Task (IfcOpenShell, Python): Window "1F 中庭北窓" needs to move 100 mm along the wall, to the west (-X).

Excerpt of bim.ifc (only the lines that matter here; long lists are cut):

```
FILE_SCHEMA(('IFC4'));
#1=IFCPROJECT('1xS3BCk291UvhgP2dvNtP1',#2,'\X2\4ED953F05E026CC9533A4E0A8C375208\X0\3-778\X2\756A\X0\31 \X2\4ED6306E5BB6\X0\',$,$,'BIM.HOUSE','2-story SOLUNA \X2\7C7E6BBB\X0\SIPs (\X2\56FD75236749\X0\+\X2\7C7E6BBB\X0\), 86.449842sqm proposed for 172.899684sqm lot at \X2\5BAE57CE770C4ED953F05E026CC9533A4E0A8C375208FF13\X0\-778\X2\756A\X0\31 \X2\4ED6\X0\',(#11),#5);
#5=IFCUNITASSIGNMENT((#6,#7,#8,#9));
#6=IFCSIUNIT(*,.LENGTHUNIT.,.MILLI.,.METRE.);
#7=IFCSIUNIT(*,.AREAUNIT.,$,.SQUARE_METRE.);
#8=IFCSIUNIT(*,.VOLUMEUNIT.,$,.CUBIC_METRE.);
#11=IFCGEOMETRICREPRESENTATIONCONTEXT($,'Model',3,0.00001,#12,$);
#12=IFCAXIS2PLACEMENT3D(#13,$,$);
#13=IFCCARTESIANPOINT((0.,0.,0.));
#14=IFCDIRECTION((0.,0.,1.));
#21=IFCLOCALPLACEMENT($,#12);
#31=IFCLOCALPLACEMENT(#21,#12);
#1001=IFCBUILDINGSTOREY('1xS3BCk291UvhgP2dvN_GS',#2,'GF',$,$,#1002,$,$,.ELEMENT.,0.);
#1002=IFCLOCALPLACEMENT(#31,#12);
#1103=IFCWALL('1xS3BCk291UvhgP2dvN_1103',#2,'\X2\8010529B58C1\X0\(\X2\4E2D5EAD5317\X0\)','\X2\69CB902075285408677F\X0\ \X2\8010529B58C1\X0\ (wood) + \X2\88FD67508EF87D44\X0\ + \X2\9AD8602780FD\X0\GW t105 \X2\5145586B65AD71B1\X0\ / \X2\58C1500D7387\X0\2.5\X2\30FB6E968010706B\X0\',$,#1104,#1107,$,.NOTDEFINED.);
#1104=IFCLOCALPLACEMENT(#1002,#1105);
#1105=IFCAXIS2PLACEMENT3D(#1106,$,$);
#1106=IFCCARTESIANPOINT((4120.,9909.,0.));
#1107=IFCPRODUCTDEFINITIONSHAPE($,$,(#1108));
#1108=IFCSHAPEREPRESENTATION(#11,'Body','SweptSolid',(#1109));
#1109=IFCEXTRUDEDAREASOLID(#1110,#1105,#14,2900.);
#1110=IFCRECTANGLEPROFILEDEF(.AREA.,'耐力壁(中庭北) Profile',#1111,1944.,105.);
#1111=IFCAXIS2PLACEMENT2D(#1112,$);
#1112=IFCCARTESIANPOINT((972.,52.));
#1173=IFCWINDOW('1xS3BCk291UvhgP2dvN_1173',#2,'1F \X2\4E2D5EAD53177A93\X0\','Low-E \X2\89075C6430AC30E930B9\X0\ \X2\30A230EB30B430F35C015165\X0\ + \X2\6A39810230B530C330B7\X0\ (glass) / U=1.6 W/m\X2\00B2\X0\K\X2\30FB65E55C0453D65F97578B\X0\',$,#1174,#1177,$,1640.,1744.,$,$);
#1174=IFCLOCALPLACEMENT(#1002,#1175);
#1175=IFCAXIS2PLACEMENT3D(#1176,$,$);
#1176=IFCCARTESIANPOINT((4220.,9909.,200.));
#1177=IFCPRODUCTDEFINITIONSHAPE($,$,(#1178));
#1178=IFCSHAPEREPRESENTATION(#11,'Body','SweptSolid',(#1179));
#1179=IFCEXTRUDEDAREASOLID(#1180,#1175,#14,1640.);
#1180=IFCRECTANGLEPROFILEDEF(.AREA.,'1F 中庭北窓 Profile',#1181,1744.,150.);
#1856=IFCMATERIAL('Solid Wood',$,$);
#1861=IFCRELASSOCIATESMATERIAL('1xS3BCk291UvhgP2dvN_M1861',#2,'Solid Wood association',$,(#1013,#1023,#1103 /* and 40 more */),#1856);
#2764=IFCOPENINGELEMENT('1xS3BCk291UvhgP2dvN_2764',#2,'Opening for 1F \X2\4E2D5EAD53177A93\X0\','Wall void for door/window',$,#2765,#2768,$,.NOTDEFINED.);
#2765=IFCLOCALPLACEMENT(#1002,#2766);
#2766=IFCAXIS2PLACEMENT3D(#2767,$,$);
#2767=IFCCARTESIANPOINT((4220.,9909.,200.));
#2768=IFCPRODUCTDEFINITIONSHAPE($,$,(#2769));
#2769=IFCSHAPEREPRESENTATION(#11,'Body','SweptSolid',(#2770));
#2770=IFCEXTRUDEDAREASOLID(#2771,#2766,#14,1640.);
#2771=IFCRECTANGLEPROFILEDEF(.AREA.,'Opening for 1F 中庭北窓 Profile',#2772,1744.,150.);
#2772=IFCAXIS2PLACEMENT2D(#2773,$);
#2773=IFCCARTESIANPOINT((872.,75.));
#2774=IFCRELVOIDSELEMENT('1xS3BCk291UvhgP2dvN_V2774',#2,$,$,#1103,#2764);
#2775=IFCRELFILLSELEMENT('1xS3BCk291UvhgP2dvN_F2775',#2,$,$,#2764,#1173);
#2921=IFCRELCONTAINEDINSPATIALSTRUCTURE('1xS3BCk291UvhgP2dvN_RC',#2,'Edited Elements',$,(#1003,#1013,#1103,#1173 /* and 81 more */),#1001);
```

```python
import ifcopenshell
import ifcopenshell.api.geometry
import ifcopenshell.util.placement
import ifcopenshell.util.unit

model = ifcopenshell.open("bim.ifc")
unit_scale = ifcopenshell.util.unit.calculate_unit_scale(model)

window = model.by_guid("1xS3BCk291UvhgP2dvN_1173")
opening = window.FillsVoids[0].RelatingOpeningElement
wall = opening.VoidsElements[0].RelatingBuildingElement

wall_matrix = ifcopenshell.util.placement.get_local_placement(wall.ObjectPlacement)
shift = wall_matrix[:3, 0] * -0.1 / unit_scale
before = ifcopenshell.util.placement.get_local_placement(window.ObjectPlacement)[:3, 3].copy()

# The window is not placed relative to its opening, so move both.
for product in (opening, window):
    matrix = ifcopenshell.util.placement.get_local_placement(product.ObjectPlacement)
    matrix[:3, 3] += shift
    ifcopenshell.api.geometry.edit_object_placement(model, product=product, matrix=matrix, is_si=False)

after = ifcopenshell.util.placement.get_local_placement(window.ObjectPlacement)[:3, 3]
print("window moved by", (after - before).round(3) + 0.0)

model.write("bim_rev.ifc")
```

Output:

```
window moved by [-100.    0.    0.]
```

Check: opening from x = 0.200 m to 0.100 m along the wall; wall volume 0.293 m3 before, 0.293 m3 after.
